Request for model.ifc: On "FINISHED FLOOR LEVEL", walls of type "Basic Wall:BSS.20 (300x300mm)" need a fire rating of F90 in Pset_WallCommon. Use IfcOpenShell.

First a look at what the model holds.

```python
import ifcopenshell
import ifcopenshell.util.element

model = ifcopenshell.open("model.ifc")
print(model.schema)
storey = next(s for s in model.by_type("IfcBuildingStorey") if s.Name == "FINISHED FLOOR LEVEL")
walls = [e for e in ifcopenshell.util.element.get_decomposition(storey) if e.is_a("IfcWall")]
seen = {}
for e in walls:
    element_type = ifcopenshell.util.element.get_type(e)
    key = (element_type.Name if element_type != e and element_type else None, ifcopenshell.util.element.get_pset(e, "Pset_WallCommon", "FireRating"))
    seen[key] = seen.get(key, 0) + 1
for (name, value), count in sorted(seen.items(), key=str):
    print(count, "x", name, "|", value)
```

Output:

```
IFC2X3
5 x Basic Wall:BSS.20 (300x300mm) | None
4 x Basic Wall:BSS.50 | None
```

```python
import ifcopenshell
import ifcopenshell.api.pset
import ifcopenshell.util.element

model = ifcopenshell.open("model.ifc")

storey = next(s for s in model.by_type("IfcBuildingStorey") if s.Name == "FINISHED FLOOR LEVEL")
walls = [e for e in ifcopenshell.util.element.get_decomposition(storey) if e.is_a("IfcWall")]

count = 0
for e in walls:
    element_type = ifcopenshell.util.element.get_type(e)
    if element_type in (None, e) or element_type.Name != "Basic Wall:BSS.20 (300x300mm)":
        continue
    # add_pset returns the element's existing set when there is one.
    pset = ifcopenshell.api.pset.add_pset(model, product=e, name="Pset_WallCommon")
    ifcopenshell.api.pset.edit_pset(model, pset=pset, properties={"FireRating": "F90"})
    count += 1

print(count, "walls updated")

model.write("model_edited.ifc")
```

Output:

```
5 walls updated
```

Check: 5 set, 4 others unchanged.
